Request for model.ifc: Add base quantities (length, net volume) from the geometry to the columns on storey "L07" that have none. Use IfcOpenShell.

First a look at what the model holds.

```python
import ifcopenshell
import ifcopenshell.util.element
import ifcopenshell.util.unit

model = ifcopenshell.open("model.ifc")
print(model.schema)
for unit_type in ("LENGTHUNIT", "AREAUNIT", "VOLUMEUNIT"):
    print(unit_type, ifcopenshell.util.unit.calculate_unit_scale(model, unit_type))
storey = next(s for s in model.by_type("IfcBuildingStorey") if s.Name == "L07")
columns = [e for e in ifcopenshell.util.element.get_decomposition(storey) if e.is_a("IfcColumn")]
for e in sorted(columns, key=lambda e: e.id()):
    print(e.id(), e.is_a(), e.Name, list(ifcopenshell.util.element.get_psets(e, qtos_only=True)), sep=" | ")
```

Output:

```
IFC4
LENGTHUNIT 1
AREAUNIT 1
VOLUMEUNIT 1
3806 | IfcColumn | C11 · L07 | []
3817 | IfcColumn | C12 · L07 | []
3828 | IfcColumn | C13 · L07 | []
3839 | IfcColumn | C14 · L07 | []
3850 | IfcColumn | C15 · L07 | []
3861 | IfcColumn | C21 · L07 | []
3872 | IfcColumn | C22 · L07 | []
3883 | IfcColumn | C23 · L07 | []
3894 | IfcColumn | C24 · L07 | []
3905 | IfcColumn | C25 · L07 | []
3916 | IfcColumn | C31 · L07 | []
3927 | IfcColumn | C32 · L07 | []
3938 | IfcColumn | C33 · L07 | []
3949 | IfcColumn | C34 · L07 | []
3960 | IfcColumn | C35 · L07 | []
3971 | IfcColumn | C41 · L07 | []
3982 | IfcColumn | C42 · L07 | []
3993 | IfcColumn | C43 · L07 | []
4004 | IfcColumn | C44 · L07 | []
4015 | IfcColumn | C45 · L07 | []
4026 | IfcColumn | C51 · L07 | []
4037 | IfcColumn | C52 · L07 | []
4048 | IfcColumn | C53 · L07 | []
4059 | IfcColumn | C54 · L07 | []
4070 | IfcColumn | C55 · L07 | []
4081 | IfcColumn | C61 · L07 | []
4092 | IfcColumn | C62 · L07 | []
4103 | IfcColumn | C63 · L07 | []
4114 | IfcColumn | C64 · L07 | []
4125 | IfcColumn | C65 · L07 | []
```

```python
import ifcopenshell
import ifcopenshell.api.pset
import ifcopenshell.geom
import ifcopenshell.util.element
import ifcopenshell.util.shape
import ifcopenshell.util.unit

model = ifcopenshell.open("model.ifc")
unit_scale = ifcopenshell.util.unit.calculate_unit_scale(model)
volume_scale = ifcopenshell.util.unit.calculate_unit_scale(model, "VOLUMEUNIT")
settings = ifcopenshell.geom.settings()

storey = next(s for s in model.by_type("IfcBuildingStorey") if s.Name == "L07")
columns = [e for e in ifcopenshell.util.element.get_decomposition(storey) if e.is_a("IfcColumn")]

for e in sorted(columns, key=lambda e: e.id()):
    if ifcopenshell.util.element.get_psets(e, qtos_only=True, should_inherit=False):
        continue
    # Geometry comes back in metres, in the element's own axes.
    shape = ifcopenshell.geom.create_shape(settings, e)
    values = {
        "Length": ifcopenshell.util.shape.get_z(shape.geometry) / unit_scale,
        "NetVolume": ifcopenshell.util.shape.get_volume(shape.geometry) / volume_scale,
    }
    qto = ifcopenshell.api.pset.add_qto(model, product=e, name="Qto_ColumnBaseQuantities")
    ifcopenshell.api.pset.edit_qto(model, qto=qto, properties=values)
    print(e.id(), {k: round(v, 3) for k, v in values.items()})

model.write("model_rev.ifc")
```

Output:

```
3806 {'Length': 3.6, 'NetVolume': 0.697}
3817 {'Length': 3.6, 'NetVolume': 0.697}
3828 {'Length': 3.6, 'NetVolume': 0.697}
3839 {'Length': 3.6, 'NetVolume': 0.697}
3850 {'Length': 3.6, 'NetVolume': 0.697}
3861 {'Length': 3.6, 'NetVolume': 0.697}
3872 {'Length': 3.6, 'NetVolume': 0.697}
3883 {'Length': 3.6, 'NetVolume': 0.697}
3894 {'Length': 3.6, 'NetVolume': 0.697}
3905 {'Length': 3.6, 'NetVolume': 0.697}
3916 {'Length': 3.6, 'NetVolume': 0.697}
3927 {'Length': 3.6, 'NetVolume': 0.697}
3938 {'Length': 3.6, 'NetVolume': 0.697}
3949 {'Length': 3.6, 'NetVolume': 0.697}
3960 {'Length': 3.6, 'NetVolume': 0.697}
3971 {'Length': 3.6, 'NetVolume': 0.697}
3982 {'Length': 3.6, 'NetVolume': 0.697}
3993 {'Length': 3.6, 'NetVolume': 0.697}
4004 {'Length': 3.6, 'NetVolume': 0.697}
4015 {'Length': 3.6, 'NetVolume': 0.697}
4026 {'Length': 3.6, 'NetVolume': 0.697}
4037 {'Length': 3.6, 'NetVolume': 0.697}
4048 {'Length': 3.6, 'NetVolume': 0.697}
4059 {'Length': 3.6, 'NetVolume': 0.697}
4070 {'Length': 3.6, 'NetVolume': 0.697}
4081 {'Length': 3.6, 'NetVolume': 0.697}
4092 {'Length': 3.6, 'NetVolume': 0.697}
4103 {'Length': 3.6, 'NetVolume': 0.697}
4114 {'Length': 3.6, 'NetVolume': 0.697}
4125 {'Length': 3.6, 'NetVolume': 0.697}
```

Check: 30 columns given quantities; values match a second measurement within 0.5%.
